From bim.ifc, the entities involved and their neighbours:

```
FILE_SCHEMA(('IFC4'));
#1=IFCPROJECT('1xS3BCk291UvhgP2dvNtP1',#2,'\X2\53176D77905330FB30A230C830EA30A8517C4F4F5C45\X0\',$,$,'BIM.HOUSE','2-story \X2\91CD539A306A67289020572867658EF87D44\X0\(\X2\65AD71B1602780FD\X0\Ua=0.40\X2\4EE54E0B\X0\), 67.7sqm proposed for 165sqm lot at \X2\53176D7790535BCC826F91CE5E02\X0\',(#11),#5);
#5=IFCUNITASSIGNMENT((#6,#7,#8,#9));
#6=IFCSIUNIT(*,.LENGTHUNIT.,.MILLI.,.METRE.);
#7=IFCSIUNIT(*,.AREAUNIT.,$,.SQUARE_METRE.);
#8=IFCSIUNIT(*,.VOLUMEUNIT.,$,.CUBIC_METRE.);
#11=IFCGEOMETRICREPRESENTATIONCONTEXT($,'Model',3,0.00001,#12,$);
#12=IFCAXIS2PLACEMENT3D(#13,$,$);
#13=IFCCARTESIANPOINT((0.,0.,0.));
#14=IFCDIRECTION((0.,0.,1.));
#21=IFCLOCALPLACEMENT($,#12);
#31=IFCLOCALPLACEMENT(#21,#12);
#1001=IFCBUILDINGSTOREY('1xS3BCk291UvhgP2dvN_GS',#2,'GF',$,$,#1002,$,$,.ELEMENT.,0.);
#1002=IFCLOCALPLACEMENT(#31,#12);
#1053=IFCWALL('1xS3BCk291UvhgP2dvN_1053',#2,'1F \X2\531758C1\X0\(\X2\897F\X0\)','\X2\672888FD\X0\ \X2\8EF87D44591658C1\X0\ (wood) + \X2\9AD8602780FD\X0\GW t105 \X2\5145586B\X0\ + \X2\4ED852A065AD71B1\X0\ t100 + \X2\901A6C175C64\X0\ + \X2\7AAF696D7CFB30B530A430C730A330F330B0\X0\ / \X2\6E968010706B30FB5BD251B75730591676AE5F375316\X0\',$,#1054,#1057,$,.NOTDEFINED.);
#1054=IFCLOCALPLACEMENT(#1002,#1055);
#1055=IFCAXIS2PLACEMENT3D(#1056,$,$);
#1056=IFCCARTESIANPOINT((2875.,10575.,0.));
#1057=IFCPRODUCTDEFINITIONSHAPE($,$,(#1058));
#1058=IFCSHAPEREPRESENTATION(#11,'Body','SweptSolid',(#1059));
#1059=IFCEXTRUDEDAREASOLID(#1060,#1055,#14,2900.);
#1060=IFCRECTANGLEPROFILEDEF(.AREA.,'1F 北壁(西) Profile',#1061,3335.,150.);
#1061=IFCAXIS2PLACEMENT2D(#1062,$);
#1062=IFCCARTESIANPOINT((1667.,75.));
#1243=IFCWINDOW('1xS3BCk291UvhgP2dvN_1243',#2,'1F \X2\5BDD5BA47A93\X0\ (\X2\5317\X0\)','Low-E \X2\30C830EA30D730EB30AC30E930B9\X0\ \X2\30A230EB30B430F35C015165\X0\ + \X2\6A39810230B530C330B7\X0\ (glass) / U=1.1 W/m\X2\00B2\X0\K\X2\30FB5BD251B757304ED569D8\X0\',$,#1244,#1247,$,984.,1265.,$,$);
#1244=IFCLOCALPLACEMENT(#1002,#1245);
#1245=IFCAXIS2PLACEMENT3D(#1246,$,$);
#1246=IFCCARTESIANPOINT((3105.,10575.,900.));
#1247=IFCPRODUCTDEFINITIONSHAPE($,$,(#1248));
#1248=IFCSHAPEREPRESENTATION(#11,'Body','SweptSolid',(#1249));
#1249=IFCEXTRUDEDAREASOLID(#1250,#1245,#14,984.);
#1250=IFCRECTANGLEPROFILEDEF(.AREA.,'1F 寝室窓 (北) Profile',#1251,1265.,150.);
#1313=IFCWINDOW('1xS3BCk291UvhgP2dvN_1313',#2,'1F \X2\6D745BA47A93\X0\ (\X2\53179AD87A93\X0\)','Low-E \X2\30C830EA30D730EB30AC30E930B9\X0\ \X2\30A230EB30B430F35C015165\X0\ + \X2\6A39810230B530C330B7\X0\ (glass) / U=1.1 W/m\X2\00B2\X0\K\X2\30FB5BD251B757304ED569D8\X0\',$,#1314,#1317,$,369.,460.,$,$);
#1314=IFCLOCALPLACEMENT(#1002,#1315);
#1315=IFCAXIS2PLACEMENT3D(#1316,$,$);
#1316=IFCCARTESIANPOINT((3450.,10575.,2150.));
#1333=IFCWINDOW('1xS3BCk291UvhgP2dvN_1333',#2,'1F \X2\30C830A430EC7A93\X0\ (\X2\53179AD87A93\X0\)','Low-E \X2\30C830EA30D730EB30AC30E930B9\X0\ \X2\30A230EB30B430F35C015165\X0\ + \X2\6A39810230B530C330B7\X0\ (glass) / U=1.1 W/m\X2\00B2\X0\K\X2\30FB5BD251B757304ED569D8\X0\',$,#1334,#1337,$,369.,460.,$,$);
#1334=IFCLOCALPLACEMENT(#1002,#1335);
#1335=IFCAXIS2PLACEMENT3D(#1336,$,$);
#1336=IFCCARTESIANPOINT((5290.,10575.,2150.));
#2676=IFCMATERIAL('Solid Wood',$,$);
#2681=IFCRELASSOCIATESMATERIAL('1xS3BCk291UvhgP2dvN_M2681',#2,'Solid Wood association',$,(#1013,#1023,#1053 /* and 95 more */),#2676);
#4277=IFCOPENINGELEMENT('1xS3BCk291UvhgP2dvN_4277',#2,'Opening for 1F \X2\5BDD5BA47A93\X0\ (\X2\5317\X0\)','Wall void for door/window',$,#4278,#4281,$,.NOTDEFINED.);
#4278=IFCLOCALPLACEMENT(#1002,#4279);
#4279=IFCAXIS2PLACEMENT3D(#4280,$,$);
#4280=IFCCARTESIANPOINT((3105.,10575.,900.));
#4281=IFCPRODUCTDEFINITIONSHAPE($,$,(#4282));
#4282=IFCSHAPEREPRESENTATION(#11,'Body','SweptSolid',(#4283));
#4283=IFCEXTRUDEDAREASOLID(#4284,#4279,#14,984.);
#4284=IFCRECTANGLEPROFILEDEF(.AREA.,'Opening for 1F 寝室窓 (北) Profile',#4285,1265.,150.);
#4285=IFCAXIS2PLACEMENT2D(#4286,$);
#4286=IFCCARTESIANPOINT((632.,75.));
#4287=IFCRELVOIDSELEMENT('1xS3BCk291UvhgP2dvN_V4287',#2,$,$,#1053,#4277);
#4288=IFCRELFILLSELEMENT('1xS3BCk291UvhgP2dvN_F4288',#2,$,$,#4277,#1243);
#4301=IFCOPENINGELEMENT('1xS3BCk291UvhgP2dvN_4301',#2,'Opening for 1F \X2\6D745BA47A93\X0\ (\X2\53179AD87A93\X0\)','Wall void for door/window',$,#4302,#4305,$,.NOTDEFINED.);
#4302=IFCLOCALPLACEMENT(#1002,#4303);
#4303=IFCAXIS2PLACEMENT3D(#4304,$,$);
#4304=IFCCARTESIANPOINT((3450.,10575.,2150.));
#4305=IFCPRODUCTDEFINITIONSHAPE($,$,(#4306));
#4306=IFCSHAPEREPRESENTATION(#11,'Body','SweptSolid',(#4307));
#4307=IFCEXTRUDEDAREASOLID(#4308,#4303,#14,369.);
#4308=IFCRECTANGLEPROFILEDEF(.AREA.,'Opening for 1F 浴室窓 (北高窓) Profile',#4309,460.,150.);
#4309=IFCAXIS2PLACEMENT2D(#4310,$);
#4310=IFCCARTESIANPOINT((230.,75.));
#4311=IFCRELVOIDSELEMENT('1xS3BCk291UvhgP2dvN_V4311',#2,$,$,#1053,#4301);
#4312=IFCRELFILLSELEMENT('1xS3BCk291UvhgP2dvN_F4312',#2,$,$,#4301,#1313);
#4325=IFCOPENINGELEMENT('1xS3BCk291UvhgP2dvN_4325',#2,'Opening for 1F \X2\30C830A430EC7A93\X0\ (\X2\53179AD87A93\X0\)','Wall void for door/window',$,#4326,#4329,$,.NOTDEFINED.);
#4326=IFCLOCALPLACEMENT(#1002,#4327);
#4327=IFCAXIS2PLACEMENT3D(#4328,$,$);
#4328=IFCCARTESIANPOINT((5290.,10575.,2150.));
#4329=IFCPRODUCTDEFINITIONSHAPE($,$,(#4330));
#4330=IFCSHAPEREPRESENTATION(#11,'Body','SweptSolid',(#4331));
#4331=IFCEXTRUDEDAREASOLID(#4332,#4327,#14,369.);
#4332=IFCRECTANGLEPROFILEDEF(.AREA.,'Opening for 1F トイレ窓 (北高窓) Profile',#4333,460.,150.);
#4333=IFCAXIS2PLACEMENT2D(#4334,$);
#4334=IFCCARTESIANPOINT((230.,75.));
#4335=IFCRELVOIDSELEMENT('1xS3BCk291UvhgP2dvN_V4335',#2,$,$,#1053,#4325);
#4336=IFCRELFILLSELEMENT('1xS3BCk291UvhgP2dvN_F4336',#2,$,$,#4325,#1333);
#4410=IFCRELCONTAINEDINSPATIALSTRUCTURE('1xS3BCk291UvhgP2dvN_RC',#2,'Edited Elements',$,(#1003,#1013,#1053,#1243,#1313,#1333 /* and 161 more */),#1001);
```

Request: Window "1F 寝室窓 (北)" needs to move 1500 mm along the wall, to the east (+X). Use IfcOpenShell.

```python
import ifcopenshell
import ifcopenshell.api.geometry
import ifcopenshell.util.placement

model = ifcopenshell.open("bim.ifc")

window = model.by_guid("1xS3BCk291UvhgP2dvN_1243")
opening = window.FillsVoids[0].RelatingOpeningElement
wall = opening.VoidsElements[0].RelatingBuildingElement

wall_matrix = ifcopenshell.util.placement.get_local_placement(wall.ObjectPlacement)
shift = wall_matrix[:3, 0] * 1500.0
before = ifcopenshell.util.placement.get_local_placement(window.ObjectPlacement)[:3, 3].copy()

# The window is not placed relative to its opening, so move both.
for product in (opening, window):
    matrix = ifcopenshell.util.placement.get_local_placement(product.ObjectPlacement)
    matrix[:3, 3] += shift
    ifcopenshell.api.geometry.edit_object_placement(model, product=product, matrix=matrix, is_si=False)

after = ifcopenshell.util.placement.get_local_placement(window.ObjectPlacement)[:3, 3]
print("window moved by", (after - before).round(3) + 0.0)

model.write("bim_updated.ifc")
```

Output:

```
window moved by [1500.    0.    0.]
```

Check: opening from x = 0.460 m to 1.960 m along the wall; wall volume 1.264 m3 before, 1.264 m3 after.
